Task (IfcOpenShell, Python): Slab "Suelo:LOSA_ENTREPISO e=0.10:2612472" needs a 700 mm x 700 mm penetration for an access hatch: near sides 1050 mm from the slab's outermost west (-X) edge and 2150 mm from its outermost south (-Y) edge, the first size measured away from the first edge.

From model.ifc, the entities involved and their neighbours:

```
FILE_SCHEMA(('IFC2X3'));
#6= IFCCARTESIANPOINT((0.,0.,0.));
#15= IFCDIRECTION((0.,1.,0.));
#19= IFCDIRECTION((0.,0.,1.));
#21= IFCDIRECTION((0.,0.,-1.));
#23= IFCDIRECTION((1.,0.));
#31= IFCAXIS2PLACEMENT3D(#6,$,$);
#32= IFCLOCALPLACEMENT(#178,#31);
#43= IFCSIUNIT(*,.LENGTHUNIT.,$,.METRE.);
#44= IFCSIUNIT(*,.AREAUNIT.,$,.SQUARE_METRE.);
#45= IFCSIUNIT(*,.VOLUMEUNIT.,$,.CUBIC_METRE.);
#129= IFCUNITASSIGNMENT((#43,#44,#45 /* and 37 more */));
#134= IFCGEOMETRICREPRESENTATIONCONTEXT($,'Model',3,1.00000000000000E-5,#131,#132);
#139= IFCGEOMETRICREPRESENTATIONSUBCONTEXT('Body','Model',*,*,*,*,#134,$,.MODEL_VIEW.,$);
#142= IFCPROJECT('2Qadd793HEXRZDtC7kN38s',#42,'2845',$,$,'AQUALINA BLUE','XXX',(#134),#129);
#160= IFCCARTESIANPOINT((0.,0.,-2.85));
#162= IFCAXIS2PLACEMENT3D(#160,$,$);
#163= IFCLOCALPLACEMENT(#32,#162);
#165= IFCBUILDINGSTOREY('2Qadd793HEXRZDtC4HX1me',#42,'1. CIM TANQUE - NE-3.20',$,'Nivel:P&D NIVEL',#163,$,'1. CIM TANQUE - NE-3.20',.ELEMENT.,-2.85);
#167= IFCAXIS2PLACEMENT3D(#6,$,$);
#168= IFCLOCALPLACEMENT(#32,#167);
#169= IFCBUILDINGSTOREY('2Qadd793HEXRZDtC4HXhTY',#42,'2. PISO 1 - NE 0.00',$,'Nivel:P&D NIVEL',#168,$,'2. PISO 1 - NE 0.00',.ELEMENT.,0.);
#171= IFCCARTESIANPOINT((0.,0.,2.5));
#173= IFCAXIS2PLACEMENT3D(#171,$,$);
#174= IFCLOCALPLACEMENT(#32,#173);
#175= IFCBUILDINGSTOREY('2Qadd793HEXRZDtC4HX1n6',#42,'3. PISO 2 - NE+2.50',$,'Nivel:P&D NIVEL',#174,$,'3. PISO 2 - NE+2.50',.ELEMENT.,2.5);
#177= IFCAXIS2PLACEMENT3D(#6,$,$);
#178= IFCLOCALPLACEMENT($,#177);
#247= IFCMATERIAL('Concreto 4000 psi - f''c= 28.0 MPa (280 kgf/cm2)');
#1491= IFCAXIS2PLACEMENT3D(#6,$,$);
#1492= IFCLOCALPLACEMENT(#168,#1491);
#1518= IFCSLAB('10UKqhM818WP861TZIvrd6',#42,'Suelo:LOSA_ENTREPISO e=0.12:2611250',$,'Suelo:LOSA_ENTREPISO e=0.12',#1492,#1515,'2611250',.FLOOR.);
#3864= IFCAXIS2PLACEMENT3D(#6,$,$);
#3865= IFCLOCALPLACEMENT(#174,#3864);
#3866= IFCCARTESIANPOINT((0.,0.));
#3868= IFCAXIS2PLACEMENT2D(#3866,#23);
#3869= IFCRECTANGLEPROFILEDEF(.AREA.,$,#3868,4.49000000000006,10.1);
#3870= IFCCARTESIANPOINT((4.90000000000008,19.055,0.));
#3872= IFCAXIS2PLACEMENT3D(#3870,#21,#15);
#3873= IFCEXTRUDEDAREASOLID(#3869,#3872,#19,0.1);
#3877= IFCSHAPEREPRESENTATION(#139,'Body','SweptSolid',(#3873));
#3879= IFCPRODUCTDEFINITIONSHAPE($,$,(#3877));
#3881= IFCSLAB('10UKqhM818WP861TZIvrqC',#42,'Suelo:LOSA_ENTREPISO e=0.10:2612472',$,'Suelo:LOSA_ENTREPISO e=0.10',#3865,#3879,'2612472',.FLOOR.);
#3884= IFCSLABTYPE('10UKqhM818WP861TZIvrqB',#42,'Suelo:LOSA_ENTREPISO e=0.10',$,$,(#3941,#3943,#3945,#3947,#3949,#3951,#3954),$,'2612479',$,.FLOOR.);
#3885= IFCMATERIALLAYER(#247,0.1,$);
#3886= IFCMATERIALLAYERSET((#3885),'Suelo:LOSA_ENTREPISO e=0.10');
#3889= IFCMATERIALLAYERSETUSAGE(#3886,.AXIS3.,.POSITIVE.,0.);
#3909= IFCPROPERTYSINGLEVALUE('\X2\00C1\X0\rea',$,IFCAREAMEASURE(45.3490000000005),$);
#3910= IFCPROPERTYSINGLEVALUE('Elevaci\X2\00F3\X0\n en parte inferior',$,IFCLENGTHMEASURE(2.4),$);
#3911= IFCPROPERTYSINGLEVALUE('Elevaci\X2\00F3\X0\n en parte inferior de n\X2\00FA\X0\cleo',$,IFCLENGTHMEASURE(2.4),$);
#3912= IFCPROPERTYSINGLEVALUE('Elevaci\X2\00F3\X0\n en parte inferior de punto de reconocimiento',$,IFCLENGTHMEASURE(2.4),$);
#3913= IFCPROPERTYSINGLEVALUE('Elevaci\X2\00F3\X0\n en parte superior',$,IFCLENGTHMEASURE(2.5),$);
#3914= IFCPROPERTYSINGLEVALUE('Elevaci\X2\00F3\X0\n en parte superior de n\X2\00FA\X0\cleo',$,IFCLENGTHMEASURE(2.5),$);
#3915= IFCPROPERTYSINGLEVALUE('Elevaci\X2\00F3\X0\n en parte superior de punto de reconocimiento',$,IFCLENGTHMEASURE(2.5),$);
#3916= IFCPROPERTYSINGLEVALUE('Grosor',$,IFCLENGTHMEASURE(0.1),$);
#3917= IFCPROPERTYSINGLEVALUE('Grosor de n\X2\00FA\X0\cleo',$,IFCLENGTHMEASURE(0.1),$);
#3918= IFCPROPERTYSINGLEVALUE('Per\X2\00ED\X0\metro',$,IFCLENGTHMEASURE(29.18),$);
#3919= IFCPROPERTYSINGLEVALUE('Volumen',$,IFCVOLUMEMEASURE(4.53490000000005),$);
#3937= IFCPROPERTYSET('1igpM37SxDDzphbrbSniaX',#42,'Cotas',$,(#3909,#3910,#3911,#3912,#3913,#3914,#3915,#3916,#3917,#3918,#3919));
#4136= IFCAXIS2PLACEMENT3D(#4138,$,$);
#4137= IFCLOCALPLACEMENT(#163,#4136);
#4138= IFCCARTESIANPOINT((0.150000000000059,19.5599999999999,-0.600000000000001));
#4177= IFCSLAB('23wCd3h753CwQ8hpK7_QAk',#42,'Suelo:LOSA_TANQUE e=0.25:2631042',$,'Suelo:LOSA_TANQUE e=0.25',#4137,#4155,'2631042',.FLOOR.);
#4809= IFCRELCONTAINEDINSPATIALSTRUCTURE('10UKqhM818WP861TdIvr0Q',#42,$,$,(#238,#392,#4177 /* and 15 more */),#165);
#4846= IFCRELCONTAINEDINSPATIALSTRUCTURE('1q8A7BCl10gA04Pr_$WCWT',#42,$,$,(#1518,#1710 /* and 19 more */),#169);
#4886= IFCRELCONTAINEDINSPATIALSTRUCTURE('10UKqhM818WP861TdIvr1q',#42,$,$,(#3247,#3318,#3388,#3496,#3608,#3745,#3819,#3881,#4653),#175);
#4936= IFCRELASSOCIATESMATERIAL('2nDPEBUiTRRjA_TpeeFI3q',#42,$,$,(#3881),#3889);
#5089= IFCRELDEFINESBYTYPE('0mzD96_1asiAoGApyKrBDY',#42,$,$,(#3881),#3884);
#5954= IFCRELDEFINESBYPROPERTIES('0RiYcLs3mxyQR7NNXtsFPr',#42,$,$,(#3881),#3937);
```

```python
import numpy as np
import ifcopenshell
import ifcopenshell.api.feature
import ifcopenshell.api.geometry
import ifcopenshell.api.pset
import ifcopenshell.api.root
import ifcopenshell.geom
import ifcopenshell.util.element
import ifcopenshell.util.placement
import ifcopenshell.util.representation
import ifcopenshell.util.shape
import ifcopenshell.util.unit

model = ifcopenshell.open("model.ifc")
unit_scale = ifcopenshell.util.unit.calculate_unit_scale(model)
area_scale = ifcopenshell.util.unit.calculate_unit_scale(model, "AREAUNIT")
volume_scale = ifcopenshell.util.unit.calculate_unit_scale(model, "VOLUMEUNIT")
settings = ifcopenshell.geom.settings()


def volume(element):
    """Net volume in cubic metres, openings subtracted."""
    shape = ifcopenshell.geom.create_shape(settings, element)
    return ifcopenshell.util.shape.get_volume(shape.geometry)


slab = model.by_guid("10UKqhM818WP861TZIvrqC")
before = volume(slab)

# Extent in the slab's own axes, in metres. The edges named are its -X and -Y sides.
slab_shape = ifcopenshell.geom.create_shape(settings, slab)
vertices = ifcopenshell.util.shape.get_vertices(slab_shape.geometry)
x_min, y_min, bottom = vertices.min(axis=0)
top = vertices[:, 2].max()

opening = ifcopenshell.api.root.create_entity(model, ifc_class="IfcOpeningElement", name="Access hatch opening")
context = ifcopenshell.util.representation.get_context(model, "Model", "Body", "MODEL_VIEW")
width, depth = 0.7, 0.7
outline = [(0.0, 0.0), (width, 0.0), (width, depth), (0.0, depth), (0.0, 0.0)]
# Overshoot both faces by 50 mm so the cut is clean.
shape = ifcopenshell.api.geometry.add_slab_representation(
    model, context=context, depth=top - bottom + 0.1, polyline=outline
)
ifcopenshell.api.geometry.assign_representation(model, product=opening, representation=shape)

matrix = ifcopenshell.util.placement.get_local_placement(slab.ObjectPlacement)
matrix[:, 3] = matrix @ np.append(np.array([x_min + 1.05, y_min + 2.15, bottom - 0.05]) / unit_scale, 1.0)
ifcopenshell.api.geometry.edit_object_placement(model, product=opening, matrix=matrix, is_si=False)
ifcopenshell.api.feature.add_feature(model, feature=opening, element=slab)

after = volume(slab)

# Update the slab's stored quantities.
pset = model.by_id(ifcopenshell.util.element.get_pset(slab, "Cotas", should_inherit=False)["id"])
ifcopenshell.api.pset.edit_pset(model, pset=pset, properties={
    "Área": model.create_entity("IfcAreaMeasure", after / (top - bottom) / area_scale),
    "Volumen": model.create_entity("IfcVolumeMeasure", after / volume_scale),
})

print(f"slab volume {before:.3f} -> {after:.3f} m3")

model.write("model_rev.ifc")
```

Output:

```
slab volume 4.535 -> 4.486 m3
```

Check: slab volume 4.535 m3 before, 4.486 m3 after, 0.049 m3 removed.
